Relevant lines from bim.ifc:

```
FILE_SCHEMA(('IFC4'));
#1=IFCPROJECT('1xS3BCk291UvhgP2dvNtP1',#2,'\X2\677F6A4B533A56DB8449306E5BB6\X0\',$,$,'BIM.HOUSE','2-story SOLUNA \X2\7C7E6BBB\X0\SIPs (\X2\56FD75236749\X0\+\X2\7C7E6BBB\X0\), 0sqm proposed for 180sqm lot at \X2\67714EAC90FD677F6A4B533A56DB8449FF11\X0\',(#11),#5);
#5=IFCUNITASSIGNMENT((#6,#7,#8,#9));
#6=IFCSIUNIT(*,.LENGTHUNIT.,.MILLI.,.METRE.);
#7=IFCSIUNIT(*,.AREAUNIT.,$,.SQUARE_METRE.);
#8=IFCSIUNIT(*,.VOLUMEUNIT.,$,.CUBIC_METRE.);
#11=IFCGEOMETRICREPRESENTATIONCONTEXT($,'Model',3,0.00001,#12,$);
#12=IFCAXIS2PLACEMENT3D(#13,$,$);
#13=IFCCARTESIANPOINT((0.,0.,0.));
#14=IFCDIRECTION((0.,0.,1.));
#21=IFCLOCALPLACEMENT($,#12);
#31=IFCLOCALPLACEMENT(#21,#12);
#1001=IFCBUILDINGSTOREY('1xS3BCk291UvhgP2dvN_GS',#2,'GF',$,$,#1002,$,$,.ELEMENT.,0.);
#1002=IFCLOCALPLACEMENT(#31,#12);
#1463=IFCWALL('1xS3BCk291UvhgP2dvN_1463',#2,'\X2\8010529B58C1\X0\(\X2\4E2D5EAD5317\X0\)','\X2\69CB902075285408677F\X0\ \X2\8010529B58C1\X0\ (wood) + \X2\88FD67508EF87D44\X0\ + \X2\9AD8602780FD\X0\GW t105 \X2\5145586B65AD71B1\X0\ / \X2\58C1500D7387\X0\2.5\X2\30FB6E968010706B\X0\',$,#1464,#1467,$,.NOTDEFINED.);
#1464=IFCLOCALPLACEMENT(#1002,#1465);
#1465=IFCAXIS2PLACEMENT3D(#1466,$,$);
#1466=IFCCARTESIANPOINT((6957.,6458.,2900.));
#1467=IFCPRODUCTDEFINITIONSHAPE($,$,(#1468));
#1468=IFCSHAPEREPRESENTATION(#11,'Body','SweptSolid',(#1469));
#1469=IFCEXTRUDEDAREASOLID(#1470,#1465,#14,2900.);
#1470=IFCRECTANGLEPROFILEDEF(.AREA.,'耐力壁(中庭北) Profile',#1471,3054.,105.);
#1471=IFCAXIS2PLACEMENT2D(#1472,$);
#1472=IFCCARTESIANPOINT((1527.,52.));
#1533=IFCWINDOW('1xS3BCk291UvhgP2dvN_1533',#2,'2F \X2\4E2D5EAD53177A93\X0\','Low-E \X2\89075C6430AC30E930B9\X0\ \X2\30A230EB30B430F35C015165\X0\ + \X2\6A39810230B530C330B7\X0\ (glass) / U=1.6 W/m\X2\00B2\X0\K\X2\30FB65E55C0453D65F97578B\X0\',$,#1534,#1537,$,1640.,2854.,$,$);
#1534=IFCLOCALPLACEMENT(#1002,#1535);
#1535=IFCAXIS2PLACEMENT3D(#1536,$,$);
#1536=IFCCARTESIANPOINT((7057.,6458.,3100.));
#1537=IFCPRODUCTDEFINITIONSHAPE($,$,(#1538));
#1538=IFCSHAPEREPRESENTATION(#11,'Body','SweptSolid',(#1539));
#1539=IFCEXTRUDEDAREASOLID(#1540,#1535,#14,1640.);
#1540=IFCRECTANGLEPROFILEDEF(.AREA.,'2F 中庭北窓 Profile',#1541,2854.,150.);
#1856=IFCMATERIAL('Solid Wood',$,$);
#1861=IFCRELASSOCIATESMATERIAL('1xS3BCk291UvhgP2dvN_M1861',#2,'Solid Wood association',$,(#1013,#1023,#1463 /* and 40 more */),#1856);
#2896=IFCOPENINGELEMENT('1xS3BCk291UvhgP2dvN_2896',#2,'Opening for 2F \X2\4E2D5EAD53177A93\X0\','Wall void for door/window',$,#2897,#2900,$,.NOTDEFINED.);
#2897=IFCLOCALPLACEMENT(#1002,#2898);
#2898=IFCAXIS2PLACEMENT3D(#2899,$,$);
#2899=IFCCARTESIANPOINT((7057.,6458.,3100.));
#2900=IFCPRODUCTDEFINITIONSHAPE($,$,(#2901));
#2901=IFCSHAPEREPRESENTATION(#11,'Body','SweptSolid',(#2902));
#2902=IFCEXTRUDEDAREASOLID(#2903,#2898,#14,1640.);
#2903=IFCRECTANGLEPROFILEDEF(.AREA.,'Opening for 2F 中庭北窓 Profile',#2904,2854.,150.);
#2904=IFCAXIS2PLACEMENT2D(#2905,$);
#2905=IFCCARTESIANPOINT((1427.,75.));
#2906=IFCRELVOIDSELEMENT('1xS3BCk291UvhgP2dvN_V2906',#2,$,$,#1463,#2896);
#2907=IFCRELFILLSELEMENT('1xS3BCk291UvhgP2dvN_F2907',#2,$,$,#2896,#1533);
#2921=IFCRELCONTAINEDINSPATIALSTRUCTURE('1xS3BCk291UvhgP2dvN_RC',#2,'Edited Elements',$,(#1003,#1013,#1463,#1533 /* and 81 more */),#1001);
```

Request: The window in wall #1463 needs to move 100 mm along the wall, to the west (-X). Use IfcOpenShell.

```python
import ifcopenshell
import ifcopenshell.api.geometry
import ifcopenshell.util.placement
import ifcopenshell.util.unit

model = ifcopenshell.open("bim.ifc")
unit_scale = ifcopenshell.util.unit.calculate_unit_scale(model)

window = model.by_guid("1xS3BCk291UvhgP2dvN_1533")
opening = window.FillsVoids[0].RelatingOpeningElement
wall = opening.VoidsElements[0].RelatingBuildingElement

wall_matrix = ifcopenshell.util.placement.get_local_placement(wall.ObjectPlacement)
shift = wall_matrix[:3, 0] * -0.1 / unit_scale
before = ifcopenshell.util.placement.get_local_placement(window.ObjectPlacement)[:3, 3].copy()

# The window is not placed relative to its opening, so move both.
for product in (opening, window):
    matrix = ifcopenshell.util.placement.get_local_placement(product.ObjectPlacement)
    matrix[:3, 3] += shift
    ifcopenshell.api.geometry.edit_object_placement(model, product=product, matrix=matrix, is_si=False)

after = ifcopenshell.util.placement.get_local_placement(window.ObjectPlacement)[:3, 3]
print("window moved by", (after - before).round(3) + 0.0)

model.write("bim_updated.ifc")
```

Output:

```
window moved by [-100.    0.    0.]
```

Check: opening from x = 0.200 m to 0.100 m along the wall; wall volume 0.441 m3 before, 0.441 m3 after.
